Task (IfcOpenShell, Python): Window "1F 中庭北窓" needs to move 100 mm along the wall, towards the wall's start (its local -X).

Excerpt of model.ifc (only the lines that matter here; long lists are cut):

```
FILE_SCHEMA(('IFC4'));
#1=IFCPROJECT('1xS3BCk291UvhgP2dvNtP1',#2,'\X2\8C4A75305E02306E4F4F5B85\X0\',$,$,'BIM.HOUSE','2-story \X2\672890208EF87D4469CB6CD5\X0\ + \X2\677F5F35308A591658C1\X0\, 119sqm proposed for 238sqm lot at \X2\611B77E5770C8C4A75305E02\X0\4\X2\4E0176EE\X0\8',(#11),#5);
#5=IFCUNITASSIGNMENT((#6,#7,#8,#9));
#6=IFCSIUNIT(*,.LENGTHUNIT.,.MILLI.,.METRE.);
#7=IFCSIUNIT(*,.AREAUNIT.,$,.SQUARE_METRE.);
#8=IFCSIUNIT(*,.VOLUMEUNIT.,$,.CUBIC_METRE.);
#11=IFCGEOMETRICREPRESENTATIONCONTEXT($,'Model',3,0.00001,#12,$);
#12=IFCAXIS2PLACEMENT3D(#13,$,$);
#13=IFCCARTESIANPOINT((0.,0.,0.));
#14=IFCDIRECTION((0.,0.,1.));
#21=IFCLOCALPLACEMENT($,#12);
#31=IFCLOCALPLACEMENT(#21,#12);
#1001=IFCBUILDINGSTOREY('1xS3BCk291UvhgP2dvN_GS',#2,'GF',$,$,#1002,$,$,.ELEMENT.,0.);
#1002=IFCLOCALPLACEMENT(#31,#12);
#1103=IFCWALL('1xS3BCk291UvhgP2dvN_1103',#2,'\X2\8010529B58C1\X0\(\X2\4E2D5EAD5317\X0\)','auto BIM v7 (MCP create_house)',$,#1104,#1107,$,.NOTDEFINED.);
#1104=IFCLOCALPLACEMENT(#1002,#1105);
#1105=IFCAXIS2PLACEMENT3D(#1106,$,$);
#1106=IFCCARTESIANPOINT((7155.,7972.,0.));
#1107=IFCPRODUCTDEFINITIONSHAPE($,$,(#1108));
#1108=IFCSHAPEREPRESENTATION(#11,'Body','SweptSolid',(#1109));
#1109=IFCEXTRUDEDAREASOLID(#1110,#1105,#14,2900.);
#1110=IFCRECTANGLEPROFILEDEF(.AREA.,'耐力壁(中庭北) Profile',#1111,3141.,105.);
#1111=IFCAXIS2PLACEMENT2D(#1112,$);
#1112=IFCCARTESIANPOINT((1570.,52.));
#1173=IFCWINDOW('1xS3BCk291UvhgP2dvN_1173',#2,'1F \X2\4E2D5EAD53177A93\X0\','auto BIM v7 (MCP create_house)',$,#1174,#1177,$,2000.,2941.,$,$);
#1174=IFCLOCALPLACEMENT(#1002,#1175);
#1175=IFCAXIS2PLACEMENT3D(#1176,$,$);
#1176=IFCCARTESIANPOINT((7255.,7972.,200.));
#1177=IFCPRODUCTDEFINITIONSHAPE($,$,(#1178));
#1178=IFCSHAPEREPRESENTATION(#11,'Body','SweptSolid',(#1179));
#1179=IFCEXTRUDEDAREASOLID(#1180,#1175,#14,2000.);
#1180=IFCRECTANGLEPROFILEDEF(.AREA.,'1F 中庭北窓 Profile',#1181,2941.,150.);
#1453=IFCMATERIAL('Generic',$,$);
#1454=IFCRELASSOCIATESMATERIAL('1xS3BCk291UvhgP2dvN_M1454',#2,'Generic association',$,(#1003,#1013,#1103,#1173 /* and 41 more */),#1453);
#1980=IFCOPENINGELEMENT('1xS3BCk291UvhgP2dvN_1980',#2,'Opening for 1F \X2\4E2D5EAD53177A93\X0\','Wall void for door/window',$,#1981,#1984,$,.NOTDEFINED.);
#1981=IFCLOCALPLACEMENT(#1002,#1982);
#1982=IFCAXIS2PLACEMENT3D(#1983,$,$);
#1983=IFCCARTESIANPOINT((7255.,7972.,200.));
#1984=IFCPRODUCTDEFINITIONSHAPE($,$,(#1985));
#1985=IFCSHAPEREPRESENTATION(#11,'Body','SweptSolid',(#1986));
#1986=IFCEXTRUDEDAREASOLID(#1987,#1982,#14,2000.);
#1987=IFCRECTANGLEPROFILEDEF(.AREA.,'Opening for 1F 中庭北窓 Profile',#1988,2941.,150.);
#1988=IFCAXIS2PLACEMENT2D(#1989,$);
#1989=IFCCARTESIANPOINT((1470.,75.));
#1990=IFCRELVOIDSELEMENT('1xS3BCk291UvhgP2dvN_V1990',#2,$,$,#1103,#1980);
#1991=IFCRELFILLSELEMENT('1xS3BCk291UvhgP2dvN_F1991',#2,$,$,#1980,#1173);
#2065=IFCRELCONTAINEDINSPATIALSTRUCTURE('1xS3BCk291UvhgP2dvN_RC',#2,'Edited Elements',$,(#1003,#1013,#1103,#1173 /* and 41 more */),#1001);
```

```python
import ifcopenshell
import ifcopenshell.api.geometry
import ifcopenshell.util.placement

model = ifcopenshell.open("model.ifc")

window = model.by_guid("1xS3BCk291UvhgP2dvN_1173")
opening = window.FillsVoids[0].RelatingOpeningElement
wall = opening.VoidsElements[0].RelatingBuildingElement

wall_matrix = ifcopenshell.util.placement.get_local_placement(wall.ObjectPlacement)
shift = wall_matrix[:3, 0] * -100.0
before = ifcopenshell.util.placement.get_local_placement(window.ObjectPlacement)[:3, 3].copy()

# The window is not placed relative to its opening, so move both.
for product in (opening, window):
    matrix = ifcopenshell.util.placement.get_local_placement(product.ObjectPlacement)
    matrix[:3, 3] += shift
    ifcopenshell.api.geometry.edit_object_placement(model, product=product, matrix=matrix, is_si=False)

after = ifcopenshell.util.placement.get_local_placement(window.ObjectPlacement)[:3, 3]
print("window moved by", (after - before).round(3) + 0.0)

model.write("model-out.ifc")
```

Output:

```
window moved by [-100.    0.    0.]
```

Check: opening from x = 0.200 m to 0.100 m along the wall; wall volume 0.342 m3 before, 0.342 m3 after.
